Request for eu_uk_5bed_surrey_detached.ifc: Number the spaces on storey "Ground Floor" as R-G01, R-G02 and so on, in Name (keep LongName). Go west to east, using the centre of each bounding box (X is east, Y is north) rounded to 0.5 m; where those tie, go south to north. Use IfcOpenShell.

First a look at what the model holds.

```python
import ifcopenshell
import ifcopenshell.util.element
import ifcopenshell.util.placement

model = ifcopenshell.open("eu_uk_5bed_surrey_detached.ifc")
print(model.schema)
storey = next(s for s in model.by_type("IfcBuildingStorey") if s.Name == "Ground Floor")
spaces = [e for e in ifcopenshell.util.element.get_decomposition(storey) if e.is_a("IfcSpace")]
for e in sorted(spaces, key=lambda e: e.id()):
    origin = ifcopenshell.util.placement.get_local_placement(e.ObjectPlacement)[:3, 3]
    print(e.id(), e.Name, e.LongName, origin.round(2) + 0.0, sep=" | ")
```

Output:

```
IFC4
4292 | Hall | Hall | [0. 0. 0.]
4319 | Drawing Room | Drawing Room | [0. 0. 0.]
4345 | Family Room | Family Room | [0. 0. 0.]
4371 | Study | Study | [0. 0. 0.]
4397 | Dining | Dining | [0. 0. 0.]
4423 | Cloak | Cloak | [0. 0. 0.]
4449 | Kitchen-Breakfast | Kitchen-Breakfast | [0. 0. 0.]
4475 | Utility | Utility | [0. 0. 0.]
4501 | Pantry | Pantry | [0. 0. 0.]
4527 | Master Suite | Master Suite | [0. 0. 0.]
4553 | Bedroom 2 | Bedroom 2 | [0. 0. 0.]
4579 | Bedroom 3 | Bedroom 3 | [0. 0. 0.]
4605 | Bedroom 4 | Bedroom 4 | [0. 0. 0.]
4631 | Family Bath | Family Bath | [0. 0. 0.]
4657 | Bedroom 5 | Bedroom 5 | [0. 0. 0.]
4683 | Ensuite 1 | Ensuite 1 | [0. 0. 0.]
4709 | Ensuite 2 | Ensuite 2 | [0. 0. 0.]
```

```python
import ifcopenshell
import ifcopenshell.geom
import ifcopenshell.util.element
import ifcopenshell.util.shape

model = ifcopenshell.open("eu_uk_5bed_surrey_detached.ifc")
settings = ifcopenshell.geom.settings()
settings.set("use-world-coords", True)


def centre(element):
    shape = ifcopenshell.geom.create_shape(settings, element)
    return ifcopenshell.util.shape.get_bbox_centroid(shape.geometry)


storey = next(s for s in model.by_type("IfcBuildingStorey") if s.Name == "Ground Floor")
spaces = [e for e in ifcopenshell.util.element.get_decomposition(storey) if e.is_a("IfcSpace")]

# Insertion points can sit at a corner or the storey origin, so sort by the geometry (in metres).
centres = {e: centre(e) for e in spaces}
spaces.sort(key=lambda e: (round(centres[e][0] / 0.5), centres[e][1]))

for i, e in enumerate(spaces, start=1):
    number = f"R-G{i:02d}"
    e.Name = number
    print(e.id(), number)

model.write("eu_uk_5bed_surrey_detached_updated.ifc")
```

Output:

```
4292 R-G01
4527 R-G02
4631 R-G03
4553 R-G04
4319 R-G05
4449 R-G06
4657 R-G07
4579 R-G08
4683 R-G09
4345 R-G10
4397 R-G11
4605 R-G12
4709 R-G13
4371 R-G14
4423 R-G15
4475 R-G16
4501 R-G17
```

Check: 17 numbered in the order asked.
